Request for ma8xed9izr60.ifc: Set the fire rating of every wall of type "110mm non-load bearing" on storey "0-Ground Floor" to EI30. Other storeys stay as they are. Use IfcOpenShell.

First a look at what the model holds.

```python
import ifcopenshell
import ifcopenshell.util.element

model = ifcopenshell.open("ma8xed9izr60.ifc")
print(model.schema)
storey = next(s for s in model.by_type("IfcBuildingStorey") if s.Name == "0-Ground Floor")
walls = [e for e in ifcopenshell.util.element.get_decomposition(storey) if e.is_a("IfcWall")]
seen = {}
for e in walls:
    element_type = ifcopenshell.util.element.get_type(e)
    key = (element_type.Name if element_type != e and element_type else None, ifcopenshell.util.element.get_pset(e, "Pset_WallCommon", "FireRating"))
    seen[key] = seen.get(key, 0) + 1
for (name, value), count in sorted(seen.items(), key=str):
    print(count, "x", name, "|", value)
```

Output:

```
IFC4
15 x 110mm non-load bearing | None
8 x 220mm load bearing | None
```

```python
import ifcopenshell
import ifcopenshell.api.pset
import ifcopenshell.util.element

model = ifcopenshell.open("ma8xed9izr60.ifc")

storey = next(s for s in model.by_type("IfcBuildingStorey") if s.Name == "0-Ground Floor")
walls = [e for e in ifcopenshell.util.element.get_decomposition(storey) if e.is_a("IfcWall")]

count = 0
for e in walls:
    element_type = ifcopenshell.util.element.get_type(e)
    if element_type in (None, e) or element_type.Name != "110mm non-load bearing":
        continue
    # add_pset returns the element's existing set when there is one.
    pset = ifcopenshell.api.pset.add_pset(model, product=e, name="Pset_WallCommon")
    ifcopenshell.api.pset.edit_pset(model, pset=pset, properties={"FireRating": "EI30"})
    count += 1

print(count, "walls updated")

model.write("ma8xed9izr60_v2.ifc")
```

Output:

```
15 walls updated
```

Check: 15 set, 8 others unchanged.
